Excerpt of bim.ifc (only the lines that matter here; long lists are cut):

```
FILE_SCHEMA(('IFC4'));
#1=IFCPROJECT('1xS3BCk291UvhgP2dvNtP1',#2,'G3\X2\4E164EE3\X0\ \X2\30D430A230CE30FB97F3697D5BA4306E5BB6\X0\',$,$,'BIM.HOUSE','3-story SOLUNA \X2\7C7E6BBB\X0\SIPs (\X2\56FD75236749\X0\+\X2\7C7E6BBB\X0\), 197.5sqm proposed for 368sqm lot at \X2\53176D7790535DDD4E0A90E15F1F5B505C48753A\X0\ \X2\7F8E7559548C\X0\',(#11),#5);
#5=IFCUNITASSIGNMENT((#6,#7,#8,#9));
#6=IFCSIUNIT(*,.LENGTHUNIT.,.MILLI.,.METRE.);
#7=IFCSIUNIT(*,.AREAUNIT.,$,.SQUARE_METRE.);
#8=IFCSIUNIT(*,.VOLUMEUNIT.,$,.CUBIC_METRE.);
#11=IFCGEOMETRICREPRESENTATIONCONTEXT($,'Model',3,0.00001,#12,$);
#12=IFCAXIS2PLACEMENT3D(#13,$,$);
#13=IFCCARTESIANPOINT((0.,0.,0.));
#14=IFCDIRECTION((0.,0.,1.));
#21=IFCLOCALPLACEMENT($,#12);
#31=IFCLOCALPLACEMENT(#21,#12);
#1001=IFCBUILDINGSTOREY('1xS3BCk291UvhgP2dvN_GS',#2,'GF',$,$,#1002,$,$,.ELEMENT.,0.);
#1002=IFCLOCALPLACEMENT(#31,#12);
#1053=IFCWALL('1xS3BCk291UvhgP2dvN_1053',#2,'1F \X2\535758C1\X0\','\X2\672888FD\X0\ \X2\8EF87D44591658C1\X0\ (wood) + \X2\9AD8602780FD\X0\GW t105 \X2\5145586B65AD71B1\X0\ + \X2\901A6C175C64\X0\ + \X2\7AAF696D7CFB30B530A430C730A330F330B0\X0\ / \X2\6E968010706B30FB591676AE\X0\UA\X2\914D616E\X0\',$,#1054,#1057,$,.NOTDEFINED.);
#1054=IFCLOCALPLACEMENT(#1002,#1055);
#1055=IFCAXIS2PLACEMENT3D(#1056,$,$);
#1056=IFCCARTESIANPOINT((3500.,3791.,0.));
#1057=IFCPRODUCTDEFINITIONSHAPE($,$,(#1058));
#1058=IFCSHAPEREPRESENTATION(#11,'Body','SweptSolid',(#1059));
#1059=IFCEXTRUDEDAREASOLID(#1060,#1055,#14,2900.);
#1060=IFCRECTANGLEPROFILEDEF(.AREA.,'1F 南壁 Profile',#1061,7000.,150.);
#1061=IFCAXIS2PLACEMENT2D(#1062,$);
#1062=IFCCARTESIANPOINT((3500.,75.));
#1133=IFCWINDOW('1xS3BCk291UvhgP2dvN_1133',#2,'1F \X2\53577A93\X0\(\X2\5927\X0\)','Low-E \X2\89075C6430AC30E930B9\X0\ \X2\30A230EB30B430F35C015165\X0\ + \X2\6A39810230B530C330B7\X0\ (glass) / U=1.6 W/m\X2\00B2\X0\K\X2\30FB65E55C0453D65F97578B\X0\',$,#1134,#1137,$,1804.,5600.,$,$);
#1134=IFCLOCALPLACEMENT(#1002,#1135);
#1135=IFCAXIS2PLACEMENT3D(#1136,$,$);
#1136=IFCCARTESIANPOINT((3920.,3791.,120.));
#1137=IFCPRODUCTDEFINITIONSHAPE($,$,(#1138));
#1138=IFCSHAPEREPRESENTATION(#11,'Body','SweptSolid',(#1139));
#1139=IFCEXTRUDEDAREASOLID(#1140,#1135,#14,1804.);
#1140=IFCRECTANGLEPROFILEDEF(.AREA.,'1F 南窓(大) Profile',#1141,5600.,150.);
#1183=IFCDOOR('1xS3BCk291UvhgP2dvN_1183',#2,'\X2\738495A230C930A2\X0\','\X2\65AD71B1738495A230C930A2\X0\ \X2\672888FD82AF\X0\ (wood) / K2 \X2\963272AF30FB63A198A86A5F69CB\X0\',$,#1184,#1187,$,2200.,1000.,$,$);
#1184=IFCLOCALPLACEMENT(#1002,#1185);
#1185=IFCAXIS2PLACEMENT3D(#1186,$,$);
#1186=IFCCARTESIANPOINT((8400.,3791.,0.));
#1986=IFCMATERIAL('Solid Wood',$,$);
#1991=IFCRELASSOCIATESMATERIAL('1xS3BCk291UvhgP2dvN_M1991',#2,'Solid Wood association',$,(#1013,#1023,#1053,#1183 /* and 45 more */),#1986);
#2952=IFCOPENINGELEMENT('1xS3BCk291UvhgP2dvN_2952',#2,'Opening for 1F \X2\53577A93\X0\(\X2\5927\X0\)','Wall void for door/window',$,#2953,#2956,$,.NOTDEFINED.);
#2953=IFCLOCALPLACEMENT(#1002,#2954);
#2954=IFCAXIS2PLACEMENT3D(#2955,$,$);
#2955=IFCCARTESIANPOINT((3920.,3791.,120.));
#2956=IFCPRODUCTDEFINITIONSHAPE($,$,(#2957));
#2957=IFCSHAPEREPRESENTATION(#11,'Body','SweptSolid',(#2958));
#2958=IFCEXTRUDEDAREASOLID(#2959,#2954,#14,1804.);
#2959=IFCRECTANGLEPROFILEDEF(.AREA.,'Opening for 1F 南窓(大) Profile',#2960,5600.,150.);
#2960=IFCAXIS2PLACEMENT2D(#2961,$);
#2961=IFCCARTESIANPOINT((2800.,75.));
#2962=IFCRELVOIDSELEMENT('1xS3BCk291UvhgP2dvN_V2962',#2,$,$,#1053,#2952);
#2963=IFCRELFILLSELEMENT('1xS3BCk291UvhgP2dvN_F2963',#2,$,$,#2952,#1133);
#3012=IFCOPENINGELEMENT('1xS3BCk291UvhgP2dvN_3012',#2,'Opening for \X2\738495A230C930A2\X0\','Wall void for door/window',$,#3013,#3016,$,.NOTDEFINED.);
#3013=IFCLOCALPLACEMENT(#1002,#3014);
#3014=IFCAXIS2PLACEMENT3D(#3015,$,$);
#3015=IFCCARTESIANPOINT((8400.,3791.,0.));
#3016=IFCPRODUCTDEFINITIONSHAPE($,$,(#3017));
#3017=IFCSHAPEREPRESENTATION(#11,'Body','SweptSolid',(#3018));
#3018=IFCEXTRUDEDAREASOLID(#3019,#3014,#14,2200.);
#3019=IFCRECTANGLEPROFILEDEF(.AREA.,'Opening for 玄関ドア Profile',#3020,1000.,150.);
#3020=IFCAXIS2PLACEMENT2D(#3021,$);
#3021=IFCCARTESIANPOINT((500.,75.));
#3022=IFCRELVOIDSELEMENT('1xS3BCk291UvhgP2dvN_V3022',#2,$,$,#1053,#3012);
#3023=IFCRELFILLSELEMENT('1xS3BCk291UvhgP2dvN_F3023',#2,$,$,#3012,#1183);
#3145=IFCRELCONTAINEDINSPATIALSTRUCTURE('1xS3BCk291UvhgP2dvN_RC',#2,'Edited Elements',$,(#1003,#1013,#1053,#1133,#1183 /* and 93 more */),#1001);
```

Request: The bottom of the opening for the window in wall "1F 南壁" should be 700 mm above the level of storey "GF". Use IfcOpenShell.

```python
import numpy as np
import ifcopenshell
import ifcopenshell.api.geometry
import ifcopenshell.geom
import ifcopenshell.util.element
import ifcopenshell.util.placement
import ifcopenshell.util.shape
import ifcopenshell.util.unit

model = ifcopenshell.open("bim.ifc")
unit_scale = ifcopenshell.util.unit.calculate_unit_scale(model)

window = model.by_guid("1xS3BCk291UvhgP2dvN_1133")
opening = window.FillsVoids[0].RelatingOpeningElement
storey = ifcopenshell.util.element.get_container(window, ifc_class="IfcBuildingStorey")
level = ifcopenshell.util.placement.get_local_placement(storey.ObjectPlacement)[2, 3]

# The opening's origin need not be at the sill, so measure its lowest point.
shape = ifcopenshell.geom.create_shape(ifcopenshell.geom.settings(), opening)
bottom = ifcopenshell.util.shape.get_shape_bottom_elevation(shape, shape.geometry) / unit_scale
dz = level + 0.7 / unit_scale - bottom

shift = np.array([0.0, 0.0, dz])
# The window is not placed relative to its opening, so move both.
for product in (opening, window):
    matrix = ifcopenshell.util.placement.get_local_placement(product.ObjectPlacement)
    matrix[:3, 3] += shift
    ifcopenshell.api.geometry.edit_object_placement(model, product=product, matrix=matrix, is_si=False)

print(f"moved by {dz * unit_scale:+.3f} m")

model.write("bim_edited.ifc")
```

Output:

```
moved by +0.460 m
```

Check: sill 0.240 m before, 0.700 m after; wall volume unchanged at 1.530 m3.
